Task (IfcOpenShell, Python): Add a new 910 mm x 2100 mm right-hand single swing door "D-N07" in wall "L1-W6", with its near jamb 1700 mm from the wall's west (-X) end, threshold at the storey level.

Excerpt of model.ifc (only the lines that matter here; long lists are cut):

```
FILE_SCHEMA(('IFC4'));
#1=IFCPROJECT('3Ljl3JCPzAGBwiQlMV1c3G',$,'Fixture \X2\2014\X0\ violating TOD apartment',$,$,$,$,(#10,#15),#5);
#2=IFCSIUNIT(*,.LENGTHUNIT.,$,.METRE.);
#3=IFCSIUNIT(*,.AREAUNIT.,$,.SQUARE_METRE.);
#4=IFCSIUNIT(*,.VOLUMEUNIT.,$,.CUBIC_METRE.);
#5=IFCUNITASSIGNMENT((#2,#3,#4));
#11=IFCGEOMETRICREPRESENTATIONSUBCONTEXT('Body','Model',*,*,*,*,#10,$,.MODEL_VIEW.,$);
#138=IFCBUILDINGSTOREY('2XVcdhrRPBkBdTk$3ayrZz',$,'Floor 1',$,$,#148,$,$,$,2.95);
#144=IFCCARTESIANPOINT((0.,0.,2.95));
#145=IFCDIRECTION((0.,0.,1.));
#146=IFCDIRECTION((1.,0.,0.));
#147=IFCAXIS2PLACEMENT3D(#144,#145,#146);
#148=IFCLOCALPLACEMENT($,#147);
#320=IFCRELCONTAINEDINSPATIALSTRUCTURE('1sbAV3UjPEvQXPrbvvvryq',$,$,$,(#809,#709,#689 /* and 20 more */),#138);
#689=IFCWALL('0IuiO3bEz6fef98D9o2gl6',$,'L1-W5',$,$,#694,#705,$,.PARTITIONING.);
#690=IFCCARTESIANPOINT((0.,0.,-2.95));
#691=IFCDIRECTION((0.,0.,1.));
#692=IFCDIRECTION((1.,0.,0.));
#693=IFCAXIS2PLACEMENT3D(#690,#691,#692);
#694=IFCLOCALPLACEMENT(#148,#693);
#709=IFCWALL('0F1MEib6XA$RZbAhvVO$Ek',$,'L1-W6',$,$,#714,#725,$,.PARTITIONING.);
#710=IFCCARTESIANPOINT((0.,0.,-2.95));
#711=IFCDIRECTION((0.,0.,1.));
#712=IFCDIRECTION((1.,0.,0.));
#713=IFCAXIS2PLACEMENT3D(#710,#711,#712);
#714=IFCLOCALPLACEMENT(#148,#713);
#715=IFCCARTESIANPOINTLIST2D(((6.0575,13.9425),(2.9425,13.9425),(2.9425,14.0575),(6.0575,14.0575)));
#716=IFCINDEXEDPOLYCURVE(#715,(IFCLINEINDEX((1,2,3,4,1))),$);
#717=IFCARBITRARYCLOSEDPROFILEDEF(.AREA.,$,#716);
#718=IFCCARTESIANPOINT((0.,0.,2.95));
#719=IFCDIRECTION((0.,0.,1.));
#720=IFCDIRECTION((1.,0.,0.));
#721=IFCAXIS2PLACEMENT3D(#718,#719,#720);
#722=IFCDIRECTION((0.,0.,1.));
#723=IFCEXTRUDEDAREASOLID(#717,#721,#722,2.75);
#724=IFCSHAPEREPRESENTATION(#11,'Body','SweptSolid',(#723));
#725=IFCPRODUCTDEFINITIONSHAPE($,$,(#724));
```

```python
import numpy as np
import ifcopenshell
import ifcopenshell.api.feature
import ifcopenshell.api.geometry
import ifcopenshell.api.root
import ifcopenshell.api.spatial
import ifcopenshell.geom
import ifcopenshell.util.element
import ifcopenshell.util.placement
import ifcopenshell.util.representation
import ifcopenshell.util.shape
import ifcopenshell.util.unit

model = ifcopenshell.open("model.ifc")
unit_scale = ifcopenshell.util.unit.calculate_unit_scale(model)
settings = ifcopenshell.geom.settings()


def volume(element):
    """Net volume in cubic metres, openings subtracted."""
    shape = ifcopenshell.geom.create_shape(settings, element)
    return ifcopenshell.util.shape.get_volume(shape.geometry)


wall = model.by_id(709)
storey = ifcopenshell.util.element.get_container(wall, ifc_class="IfcBuildingStorey")
context = ifcopenshell.util.representation.get_context(model, "Model", "Body", "MODEL_VIEW")
before = volume(wall)

width, height, from_end, sill = 0.91, 2.1, 1.7, 0.0  # metres

# The wall runs along its own X axis, and the end named is its -X end.
wall_shape = ifcopenshell.geom.create_shape(settings, wall)
x, y, z = ifcopenshell.util.shape.get_vertices(wall_shape.geometry).T
start = x.min() + from_end
face, thickness = float(y.min()), float(y.max() - y.min())
wall_matrix = ifcopenshell.util.placement.get_local_placement(wall.ObjectPlacement)
level = ifcopenshell.util.placement.get_local_placement(storey.ObjectPlacement)[2, 3]


def in_wall(x, y):
    """Placement at x, y metres in the wall's axes, at sill height."""
    matrix = wall_matrix.copy()
    matrix[:, 3] = wall_matrix @ np.array([x / unit_scale, y / unit_scale, 0.0, 1.0])
    matrix[2, 3] = level + sill / unit_scale
    return matrix


# Opening: a box that overshoots both wall faces by 50 mm.
opening = ifcopenshell.api.root.create_entity(model, ifc_class="IfcOpeningElement", predefined_type="OPENING")
box = ifcopenshell.api.geometry.add_wall_representation(
    model, context=context, length=width, height=height, thickness=thickness + 0.1
)
ifcopenshell.api.geometry.assign_representation(model, product=opening, representation=box)
ifcopenshell.api.geometry.edit_object_placement(model, product=opening, matrix=in_wall(start, face - 0.05), is_si=False)
ifcopenshell.api.feature.add_feature(model, feature=opening, element=wall)

door = ifcopenshell.api.root.create_entity(model, ifc_class="IfcDoor", name="D-N07", predefined_type="DOOR")
door.OverallWidth, door.OverallHeight = width / unit_scale, height / unit_scale
door.OperationType = "SINGLE_SWING_RIGHT"
body = ifcopenshell.api.geometry.add_door_representation(
    model,
    context=context,
    overall_width=door.OverallWidth,
    overall_height=door.OverallHeight,
    operation_type="SINGLE_SWING_RIGHT",
    lining_properties={"LiningDepth": thickness / unit_scale, "ThresholdDepth": thickness / unit_scale},
)
ifcopenshell.api.geometry.assign_representation(model, product=door, representation=body)
ifcopenshell.api.spatial.assign_container(model, products=[door], relating_structure=storey)
ifcopenshell.api.feature.add_filling(model, opening=opening, element=door)

# The lining spans the wall, so the door starts at the wall face.
ifcopenshell.api.geometry.edit_object_placement(model, product=door, matrix=in_wall(start, face), is_si=False)

after = volume(wall)

print(f"wall volume {before:.3f} -> {after:.3f} m3")

model.write("model-out.ifc")
```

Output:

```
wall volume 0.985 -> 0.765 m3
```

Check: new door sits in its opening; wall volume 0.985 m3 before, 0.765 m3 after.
